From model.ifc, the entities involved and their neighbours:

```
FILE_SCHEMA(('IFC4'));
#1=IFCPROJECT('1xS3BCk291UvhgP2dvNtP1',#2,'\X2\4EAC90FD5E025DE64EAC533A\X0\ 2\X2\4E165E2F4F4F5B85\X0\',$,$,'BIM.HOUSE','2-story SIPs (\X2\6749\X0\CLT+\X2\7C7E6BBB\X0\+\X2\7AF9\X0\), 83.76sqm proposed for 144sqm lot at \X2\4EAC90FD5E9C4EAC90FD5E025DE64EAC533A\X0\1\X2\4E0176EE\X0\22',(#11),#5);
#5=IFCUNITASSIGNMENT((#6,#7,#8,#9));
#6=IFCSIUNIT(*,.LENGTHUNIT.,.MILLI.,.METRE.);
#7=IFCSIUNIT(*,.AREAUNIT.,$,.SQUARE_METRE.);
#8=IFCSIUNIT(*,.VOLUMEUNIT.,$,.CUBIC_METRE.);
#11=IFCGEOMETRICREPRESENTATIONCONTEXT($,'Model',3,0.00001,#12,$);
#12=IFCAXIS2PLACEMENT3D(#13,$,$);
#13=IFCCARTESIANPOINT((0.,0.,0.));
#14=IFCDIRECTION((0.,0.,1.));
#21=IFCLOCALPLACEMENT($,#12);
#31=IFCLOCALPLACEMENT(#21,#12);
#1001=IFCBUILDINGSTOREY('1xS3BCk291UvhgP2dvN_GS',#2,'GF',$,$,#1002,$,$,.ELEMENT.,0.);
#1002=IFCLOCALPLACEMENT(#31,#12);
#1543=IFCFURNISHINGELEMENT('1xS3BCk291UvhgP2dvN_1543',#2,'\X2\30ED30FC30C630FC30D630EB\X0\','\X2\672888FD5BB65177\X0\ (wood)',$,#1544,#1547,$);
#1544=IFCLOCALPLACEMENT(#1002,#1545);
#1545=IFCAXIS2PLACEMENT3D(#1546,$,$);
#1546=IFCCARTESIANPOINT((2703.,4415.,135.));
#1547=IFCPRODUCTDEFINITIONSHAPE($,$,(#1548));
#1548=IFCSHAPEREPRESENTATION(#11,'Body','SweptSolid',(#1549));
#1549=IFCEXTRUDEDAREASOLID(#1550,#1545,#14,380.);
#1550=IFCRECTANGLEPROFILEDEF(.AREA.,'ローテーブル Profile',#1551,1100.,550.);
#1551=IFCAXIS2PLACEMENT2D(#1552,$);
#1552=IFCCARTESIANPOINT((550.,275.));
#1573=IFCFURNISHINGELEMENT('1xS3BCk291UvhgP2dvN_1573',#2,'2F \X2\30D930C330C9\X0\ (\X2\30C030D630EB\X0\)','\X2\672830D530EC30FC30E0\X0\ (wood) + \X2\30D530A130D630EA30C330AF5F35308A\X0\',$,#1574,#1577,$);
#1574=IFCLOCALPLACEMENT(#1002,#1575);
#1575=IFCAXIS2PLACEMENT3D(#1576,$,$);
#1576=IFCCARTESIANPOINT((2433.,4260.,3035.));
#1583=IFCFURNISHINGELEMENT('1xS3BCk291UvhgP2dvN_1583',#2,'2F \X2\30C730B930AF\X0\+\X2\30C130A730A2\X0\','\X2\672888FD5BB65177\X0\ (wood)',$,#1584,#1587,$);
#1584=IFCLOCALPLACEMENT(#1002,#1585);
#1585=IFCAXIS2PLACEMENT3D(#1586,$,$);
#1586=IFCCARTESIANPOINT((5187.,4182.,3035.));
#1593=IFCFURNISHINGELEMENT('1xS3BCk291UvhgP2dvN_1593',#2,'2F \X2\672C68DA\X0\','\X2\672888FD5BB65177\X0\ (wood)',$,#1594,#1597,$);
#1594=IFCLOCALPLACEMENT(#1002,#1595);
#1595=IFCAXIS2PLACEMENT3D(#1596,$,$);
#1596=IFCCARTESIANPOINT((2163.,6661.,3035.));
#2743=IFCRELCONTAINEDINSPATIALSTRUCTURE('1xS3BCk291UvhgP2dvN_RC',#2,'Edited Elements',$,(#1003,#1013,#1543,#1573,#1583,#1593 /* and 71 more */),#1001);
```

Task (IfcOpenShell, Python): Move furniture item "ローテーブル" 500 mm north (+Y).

```python
import ifcopenshell
import ifcopenshell.api.geometry
import ifcopenshell.util.placement
import ifcopenshell.util.unit

model = ifcopenshell.open("model.ifc")
unit_scale = ifcopenshell.util.unit.calculate_unit_scale(model)

item = model.by_guid("1xS3BCk291UvhgP2dvN_1543")
matrix = ifcopenshell.util.placement.get_local_placement(item.ObjectPlacement)
matrix[1, 3] += 0.5 / unit_scale
ifcopenshell.api.geometry.edit_object_placement(model, product=item, matrix=matrix, is_si=False)

print(ifcopenshell.util.placement.get_local_placement(item.ObjectPlacement).round(3) + 0.0)

model.write("model_v2.ifc")
```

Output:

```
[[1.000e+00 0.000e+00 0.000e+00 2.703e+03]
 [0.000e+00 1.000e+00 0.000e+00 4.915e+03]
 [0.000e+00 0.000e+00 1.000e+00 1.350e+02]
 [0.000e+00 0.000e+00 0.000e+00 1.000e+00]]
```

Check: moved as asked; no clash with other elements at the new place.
